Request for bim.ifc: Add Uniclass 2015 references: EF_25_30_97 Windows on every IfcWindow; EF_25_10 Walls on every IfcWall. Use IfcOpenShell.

First a look at what the model holds.

```python
import ifcopenshell

model = ifcopenshell.open("bim.ifc")
print(model.schema)
print("classifications:", [c.Name for c in model.by_type("IfcClassification")])
for ifc_class in ("IfcDoor", "IfcRoof", "IfcStair", "IfcWall", "IfcWindow"):
    print(ifc_class, len(model.by_type(ifc_class)))
```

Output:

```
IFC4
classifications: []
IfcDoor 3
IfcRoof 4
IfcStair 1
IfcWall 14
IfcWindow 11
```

```python
import ifcopenshell
import ifcopenshell.api.classification

model = ifcopenshell.open("bim.ifc")

system = ifcopenshell.api.classification.add_classification(model, classification="Uniclass 2015")

codes = {
    "IfcWindow": ("EF_25_30_97", "Windows"),
    "IfcWall": ("EF_25_10", "Walls"),
}
for ifc_class, (code, name) in codes.items():
    products = model.by_type(ifc_class)
    ifcopenshell.api.classification.add_reference(
        model, products=products, classification=system, identification=code, name=name
    )
    print(code, len(products))

model.write("bim_edited.ifc")
```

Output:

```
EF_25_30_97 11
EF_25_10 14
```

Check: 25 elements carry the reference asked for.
